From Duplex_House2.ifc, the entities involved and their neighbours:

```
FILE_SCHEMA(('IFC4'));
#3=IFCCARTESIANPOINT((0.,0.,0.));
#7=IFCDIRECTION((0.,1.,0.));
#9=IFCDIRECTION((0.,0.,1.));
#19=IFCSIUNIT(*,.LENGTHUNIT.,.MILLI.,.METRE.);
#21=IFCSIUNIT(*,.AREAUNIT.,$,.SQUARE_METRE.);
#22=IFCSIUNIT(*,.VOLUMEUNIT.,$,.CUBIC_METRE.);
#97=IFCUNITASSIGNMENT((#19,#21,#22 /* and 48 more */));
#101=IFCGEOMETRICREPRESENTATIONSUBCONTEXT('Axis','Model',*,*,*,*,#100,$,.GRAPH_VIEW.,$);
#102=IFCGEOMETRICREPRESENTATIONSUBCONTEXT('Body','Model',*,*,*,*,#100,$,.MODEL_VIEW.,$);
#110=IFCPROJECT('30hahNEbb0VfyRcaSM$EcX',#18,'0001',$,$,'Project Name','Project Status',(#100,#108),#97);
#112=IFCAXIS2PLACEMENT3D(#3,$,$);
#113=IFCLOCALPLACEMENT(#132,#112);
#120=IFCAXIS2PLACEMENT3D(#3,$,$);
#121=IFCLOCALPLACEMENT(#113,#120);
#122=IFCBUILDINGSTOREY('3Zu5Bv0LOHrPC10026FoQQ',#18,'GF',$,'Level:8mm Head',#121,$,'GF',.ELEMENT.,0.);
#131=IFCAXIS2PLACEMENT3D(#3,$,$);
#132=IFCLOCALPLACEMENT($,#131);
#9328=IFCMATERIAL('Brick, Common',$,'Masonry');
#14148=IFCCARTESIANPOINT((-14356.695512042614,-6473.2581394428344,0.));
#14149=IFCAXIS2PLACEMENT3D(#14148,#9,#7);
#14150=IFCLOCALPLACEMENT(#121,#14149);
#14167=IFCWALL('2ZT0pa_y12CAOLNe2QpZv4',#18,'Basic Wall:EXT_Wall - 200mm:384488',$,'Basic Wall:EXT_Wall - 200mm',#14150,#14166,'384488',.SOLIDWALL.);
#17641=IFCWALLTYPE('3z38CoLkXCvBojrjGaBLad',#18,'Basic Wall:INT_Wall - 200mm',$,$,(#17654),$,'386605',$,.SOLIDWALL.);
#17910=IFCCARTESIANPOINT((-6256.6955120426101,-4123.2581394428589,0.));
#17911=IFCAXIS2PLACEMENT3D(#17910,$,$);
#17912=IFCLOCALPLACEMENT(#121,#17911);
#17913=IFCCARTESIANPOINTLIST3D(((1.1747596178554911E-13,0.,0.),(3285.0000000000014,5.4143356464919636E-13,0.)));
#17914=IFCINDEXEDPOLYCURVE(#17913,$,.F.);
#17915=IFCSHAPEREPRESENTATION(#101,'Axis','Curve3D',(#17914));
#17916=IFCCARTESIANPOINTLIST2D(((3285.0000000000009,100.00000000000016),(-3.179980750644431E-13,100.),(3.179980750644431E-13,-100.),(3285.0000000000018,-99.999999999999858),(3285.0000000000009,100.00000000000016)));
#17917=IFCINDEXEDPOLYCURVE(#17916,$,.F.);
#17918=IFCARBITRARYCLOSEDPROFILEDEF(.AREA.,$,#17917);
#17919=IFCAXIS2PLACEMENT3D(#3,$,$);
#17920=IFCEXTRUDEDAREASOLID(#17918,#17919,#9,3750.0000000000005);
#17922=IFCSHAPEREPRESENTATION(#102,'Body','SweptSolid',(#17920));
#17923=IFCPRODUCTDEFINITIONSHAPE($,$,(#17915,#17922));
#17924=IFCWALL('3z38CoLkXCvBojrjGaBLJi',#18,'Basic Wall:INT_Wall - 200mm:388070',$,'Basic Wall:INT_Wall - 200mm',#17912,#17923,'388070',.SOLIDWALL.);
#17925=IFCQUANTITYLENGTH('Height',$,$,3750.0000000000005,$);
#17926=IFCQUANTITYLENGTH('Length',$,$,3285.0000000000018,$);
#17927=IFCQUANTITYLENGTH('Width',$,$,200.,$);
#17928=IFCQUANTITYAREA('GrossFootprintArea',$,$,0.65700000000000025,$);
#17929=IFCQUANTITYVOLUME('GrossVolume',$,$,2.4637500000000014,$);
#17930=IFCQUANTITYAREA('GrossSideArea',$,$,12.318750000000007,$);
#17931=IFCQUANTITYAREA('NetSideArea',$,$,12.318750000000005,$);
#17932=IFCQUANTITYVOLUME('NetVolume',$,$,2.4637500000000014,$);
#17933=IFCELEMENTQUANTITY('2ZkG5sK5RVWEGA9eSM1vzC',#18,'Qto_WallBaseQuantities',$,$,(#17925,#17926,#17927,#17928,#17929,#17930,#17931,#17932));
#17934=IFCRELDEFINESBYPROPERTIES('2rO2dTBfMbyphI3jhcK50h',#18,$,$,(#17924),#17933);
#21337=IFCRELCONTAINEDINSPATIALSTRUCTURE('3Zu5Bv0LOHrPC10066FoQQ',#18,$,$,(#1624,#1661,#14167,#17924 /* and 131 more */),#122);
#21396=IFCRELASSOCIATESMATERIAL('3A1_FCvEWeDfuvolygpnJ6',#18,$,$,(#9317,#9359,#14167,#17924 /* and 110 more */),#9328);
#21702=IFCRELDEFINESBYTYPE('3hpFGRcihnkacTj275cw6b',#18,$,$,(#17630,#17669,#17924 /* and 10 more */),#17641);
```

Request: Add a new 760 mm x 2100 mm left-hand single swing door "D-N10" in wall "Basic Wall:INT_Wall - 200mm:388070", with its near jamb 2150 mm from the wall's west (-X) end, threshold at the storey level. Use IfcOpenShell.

```python
import numpy as np
import ifcopenshell
import ifcopenshell.api.feature
import ifcopenshell.api.geometry
import ifcopenshell.api.pset
import ifcopenshell.api.root
import ifcopenshell.api.spatial
import ifcopenshell.geom
import ifcopenshell.util.element
import ifcopenshell.util.placement
import ifcopenshell.util.representation
import ifcopenshell.util.shape
import ifcopenshell.util.unit

model = ifcopenshell.open("Duplex_House2.ifc")
unit_scale = ifcopenshell.util.unit.calculate_unit_scale(model)
area_scale = ifcopenshell.util.unit.calculate_unit_scale(model, "AREAUNIT")
volume_scale = ifcopenshell.util.unit.calculate_unit_scale(model, "VOLUMEUNIT")
settings = ifcopenshell.geom.settings()


def volume(element):
    """Net volume in cubic metres, openings subtracted."""
    shape = ifcopenshell.geom.create_shape(settings, element)
    return ifcopenshell.util.shape.get_volume(shape.geometry)


wall = model.by_guid("3z38CoLkXCvBojrjGaBLJi")
storey = ifcopenshell.util.element.get_container(wall, ifc_class="IfcBuildingStorey")
context = ifcopenshell.util.representation.get_context(model, "Model", "Body", "MODEL_VIEW")
before = volume(wall)

width, height, from_end, sill = 0.76, 2.1, 2.15, 0.0  # metres

# The wall runs along its own X axis, and the end named is its -X end.
wall_shape = ifcopenshell.geom.create_shape(settings, wall)
x, y, z = ifcopenshell.util.shape.get_vertices(wall_shape.geometry).T
start = x.min() + from_end
face, thickness = float(y.min()), float(y.max() - y.min())
wall_matrix = ifcopenshell.util.placement.get_local_placement(wall.ObjectPlacement)
level = ifcopenshell.util.placement.get_local_placement(storey.ObjectPlacement)[2, 3]


def in_wall(x, y):
    """Placement at x, y metres in the wall's axes, at sill height."""
    matrix = wall_matrix.copy()
    matrix[:, 3] = wall_matrix @ np.array([x / unit_scale, y / unit_scale, 0.0, 1.0])
    matrix[2, 3] = level + sill / unit_scale
    return matrix


# Opening: a box that overshoots both wall faces by 50 mm.
opening = ifcopenshell.api.root.create_entity(model, ifc_class="IfcOpeningElement", predefined_type="OPENING")
box = ifcopenshell.api.geometry.add_wall_representation(
    model, context=context, length=width, height=height, thickness=thickness + 0.1
)
ifcopenshell.api.geometry.assign_representation(model, product=opening, representation=box)
ifcopenshell.api.geometry.edit_object_placement(model, product=opening, matrix=in_wall(start, face - 0.05), is_si=False)
ifcopenshell.api.feature.add_feature(model, feature=opening, element=wall)

door = ifcopenshell.api.root.create_entity(model, ifc_class="IfcDoor", name="D-N10", predefined_type="DOOR")
door.OverallWidth, door.OverallHeight = width / unit_scale, height / unit_scale
door.OperationType = "SINGLE_SWING_LEFT"
body = ifcopenshell.api.geometry.add_door_representation(
    model,
    context=context,
    overall_width=door.OverallWidth,
    overall_height=door.OverallHeight,
    operation_type="SINGLE_SWING_LEFT",
    lining_properties={"LiningDepth": thickness / unit_scale, "ThresholdDepth": thickness / unit_scale},
)
ifcopenshell.api.geometry.assign_representation(model, product=door, representation=body)
ifcopenshell.api.spatial.assign_container(model, products=[door], relating_structure=storey)
ifcopenshell.api.feature.add_filling(model, opening=opening, element=door)

# The lining spans the wall, so the door starts at the wall face.
ifcopenshell.api.geometry.edit_object_placement(model, product=door, matrix=in_wall(start, face), is_si=False)

after = volume(wall)

# Update the wall's stored quantities.
qto = model.by_id(ifcopenshell.util.element.get_pset(wall, "Qto_WallBaseQuantities", should_inherit=False)["id"])
ifcopenshell.api.pset.edit_qto(model, qto=qto, properties={
    "NetSideArea": after / thickness / area_scale,
    "NetVolume": after / volume_scale,
})

print(f"wall volume {before:.3f} -> {after:.3f} m3")

model.write("Duplex_House2_updated.ifc")
```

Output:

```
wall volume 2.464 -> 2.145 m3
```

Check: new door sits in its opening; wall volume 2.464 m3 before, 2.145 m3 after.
